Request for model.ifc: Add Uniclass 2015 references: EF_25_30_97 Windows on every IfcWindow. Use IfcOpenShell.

First a look at what the model holds.

```python
import ifcopenshell

model = ifcopenshell.open("model.ifc")
print(model.schema)
print("classifications:", [c.Name for c in model.by_type("IfcClassification")])
for ifc_class in ("IfcDoor", "IfcRoof", "IfcStair", "IfcWall", "IfcWindow"):
    print(ifc_class, len(model.by_type(ifc_class)))
```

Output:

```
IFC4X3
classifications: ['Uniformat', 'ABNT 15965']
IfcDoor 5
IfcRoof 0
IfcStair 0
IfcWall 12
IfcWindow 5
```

```python
import ifcopenshell
import ifcopenshell.api.classification

model = ifcopenshell.open("model.ifc")

system = ifcopenshell.api.classification.add_classification(model, classification="Uniclass 2015")

codes = {
    "IfcWindow": ("EF_25_30_97", "Windows"),
}
for ifc_class, (code, name) in codes.items():
    products = model.by_type(ifc_class)
    ifcopenshell.api.classification.add_reference(
        model, products=products, classification=system, identification=code, name=name
    )
    print(code, len(products))

model.write("model_v2.ifc")
```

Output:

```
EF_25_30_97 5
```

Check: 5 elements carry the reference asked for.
